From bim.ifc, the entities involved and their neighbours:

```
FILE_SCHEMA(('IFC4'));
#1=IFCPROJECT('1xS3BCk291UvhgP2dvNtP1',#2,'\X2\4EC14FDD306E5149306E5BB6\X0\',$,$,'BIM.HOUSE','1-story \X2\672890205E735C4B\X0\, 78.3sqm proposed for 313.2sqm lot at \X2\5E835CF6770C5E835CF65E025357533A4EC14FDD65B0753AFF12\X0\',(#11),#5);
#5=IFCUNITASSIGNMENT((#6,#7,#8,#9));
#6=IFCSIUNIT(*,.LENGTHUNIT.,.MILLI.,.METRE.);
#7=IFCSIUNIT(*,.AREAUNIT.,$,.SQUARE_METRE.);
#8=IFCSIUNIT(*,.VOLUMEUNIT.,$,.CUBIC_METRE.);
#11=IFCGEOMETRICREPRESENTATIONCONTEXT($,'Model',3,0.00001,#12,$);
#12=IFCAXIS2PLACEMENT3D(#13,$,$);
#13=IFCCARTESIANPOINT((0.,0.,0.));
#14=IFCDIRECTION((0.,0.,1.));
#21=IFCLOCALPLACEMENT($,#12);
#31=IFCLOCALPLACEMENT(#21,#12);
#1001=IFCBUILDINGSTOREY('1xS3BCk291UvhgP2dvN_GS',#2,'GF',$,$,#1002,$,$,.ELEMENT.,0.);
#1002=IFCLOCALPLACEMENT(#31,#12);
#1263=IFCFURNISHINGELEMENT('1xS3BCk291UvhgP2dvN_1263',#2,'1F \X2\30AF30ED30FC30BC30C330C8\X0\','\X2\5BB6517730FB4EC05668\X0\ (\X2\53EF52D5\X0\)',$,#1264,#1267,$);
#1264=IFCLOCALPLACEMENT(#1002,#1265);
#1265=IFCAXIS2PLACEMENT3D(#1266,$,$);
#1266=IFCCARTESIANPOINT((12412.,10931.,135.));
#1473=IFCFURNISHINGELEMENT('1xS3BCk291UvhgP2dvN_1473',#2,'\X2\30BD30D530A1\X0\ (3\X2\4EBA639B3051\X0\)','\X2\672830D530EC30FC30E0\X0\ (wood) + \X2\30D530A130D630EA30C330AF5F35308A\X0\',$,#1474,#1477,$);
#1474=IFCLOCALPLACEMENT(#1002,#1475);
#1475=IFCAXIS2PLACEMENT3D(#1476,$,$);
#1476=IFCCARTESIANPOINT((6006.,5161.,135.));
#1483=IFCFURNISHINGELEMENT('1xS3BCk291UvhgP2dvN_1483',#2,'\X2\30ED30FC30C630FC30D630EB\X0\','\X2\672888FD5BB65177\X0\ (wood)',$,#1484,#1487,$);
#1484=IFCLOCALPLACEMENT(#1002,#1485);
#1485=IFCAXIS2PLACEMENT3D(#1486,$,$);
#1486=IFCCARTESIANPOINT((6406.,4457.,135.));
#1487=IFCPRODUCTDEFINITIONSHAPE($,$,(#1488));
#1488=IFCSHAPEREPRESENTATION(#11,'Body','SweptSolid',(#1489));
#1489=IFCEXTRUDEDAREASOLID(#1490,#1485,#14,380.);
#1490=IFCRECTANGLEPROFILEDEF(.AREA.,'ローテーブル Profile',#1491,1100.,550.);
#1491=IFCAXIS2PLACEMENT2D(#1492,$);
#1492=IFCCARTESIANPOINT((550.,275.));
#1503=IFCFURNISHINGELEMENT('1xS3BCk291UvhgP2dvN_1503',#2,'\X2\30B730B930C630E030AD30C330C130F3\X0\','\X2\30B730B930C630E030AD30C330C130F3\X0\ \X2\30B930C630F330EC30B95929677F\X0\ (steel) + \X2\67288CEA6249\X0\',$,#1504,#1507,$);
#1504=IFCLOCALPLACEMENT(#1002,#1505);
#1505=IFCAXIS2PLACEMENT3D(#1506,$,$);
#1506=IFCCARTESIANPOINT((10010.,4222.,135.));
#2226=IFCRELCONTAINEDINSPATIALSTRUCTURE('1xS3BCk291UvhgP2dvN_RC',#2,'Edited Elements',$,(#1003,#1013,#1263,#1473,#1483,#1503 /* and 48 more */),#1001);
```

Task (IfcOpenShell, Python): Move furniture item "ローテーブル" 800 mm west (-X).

```python
import ifcopenshell
import ifcopenshell.api.geometry
import ifcopenshell.util.placement
import ifcopenshell.util.unit

model = ifcopenshell.open("bim.ifc")
unit_scale = ifcopenshell.util.unit.calculate_unit_scale(model)

item = model.by_guid("1xS3BCk291UvhgP2dvN_1483")
matrix = ifcopenshell.util.placement.get_local_placement(item.ObjectPlacement)
matrix[0, 3] -= 0.8 / unit_scale
ifcopenshell.api.geometry.edit_object_placement(model, product=item, matrix=matrix, is_si=False)

print(ifcopenshell.util.placement.get_local_placement(item.ObjectPlacement).round(3) + 0.0)

model.write("bim_updated.ifc")
```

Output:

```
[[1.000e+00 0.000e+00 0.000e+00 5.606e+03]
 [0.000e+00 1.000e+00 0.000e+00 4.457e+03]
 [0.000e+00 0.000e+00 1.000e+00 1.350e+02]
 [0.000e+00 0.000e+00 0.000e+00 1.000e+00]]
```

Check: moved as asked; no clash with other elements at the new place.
